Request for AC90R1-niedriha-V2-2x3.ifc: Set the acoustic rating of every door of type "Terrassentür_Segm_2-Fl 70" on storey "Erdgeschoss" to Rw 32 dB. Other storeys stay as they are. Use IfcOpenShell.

First a look at what the model holds.

```python
import ifcopenshell
import ifcopenshell.util.element

model = ifcopenshell.open("AC90R1-niedriha-V2-2x3.ifc")
print(model.schema)
storey = next(s for s in model.by_type("IfcBuildingStorey") if s.Name == "Erdgeschoss")
doors = [e for e in ifcopenshell.util.element.get_decomposition(storey) if e.is_a("IfcDoor")]
seen = {}
for e in doors:
    element_type = ifcopenshell.util.element.get_type(e)
    key = (element_type.Name if element_type != e and element_type else None, ifcopenshell.util.element.get_pset(e, "Pset_DoorCommon", "AcousticRating"))
    seen[key] = seen.get(key, 0) + 1
for (name, value), count in sorted(seen.items(), key=str):
    print(count, "x", name, "|", value)
```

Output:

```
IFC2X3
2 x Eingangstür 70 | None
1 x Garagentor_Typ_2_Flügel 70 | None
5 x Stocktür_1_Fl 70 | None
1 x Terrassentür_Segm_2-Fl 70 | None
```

```python
import ifcopenshell
import ifcopenshell.api.pset
import ifcopenshell.util.element

model = ifcopenshell.open("AC90R1-niedriha-V2-2x3.ifc")

storey = next(s for s in model.by_type("IfcBuildingStorey") if s.Name == "Erdgeschoss")
doors = [e for e in ifcopenshell.util.element.get_decomposition(storey) if e.is_a("IfcDoor")]

count = 0
for e in doors:
    element_type = ifcopenshell.util.element.get_type(e)
    if element_type in (None, e) or element_type.Name != "Terrassentür_Segm_2-Fl 70":
        continue
    # add_pset returns the element's existing set when there is one.
    pset = ifcopenshell.api.pset.add_pset(model, product=e, name="Pset_DoorCommon")
    ifcopenshell.api.pset.edit_pset(model, pset=pset, properties={"AcousticRating": "Rw 32 dB"})
    count += 1

print(count, "doors updated")

model.write("AC90R1-niedriha-V2-2x3_edited.ifc")
```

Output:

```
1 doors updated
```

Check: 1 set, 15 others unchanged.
